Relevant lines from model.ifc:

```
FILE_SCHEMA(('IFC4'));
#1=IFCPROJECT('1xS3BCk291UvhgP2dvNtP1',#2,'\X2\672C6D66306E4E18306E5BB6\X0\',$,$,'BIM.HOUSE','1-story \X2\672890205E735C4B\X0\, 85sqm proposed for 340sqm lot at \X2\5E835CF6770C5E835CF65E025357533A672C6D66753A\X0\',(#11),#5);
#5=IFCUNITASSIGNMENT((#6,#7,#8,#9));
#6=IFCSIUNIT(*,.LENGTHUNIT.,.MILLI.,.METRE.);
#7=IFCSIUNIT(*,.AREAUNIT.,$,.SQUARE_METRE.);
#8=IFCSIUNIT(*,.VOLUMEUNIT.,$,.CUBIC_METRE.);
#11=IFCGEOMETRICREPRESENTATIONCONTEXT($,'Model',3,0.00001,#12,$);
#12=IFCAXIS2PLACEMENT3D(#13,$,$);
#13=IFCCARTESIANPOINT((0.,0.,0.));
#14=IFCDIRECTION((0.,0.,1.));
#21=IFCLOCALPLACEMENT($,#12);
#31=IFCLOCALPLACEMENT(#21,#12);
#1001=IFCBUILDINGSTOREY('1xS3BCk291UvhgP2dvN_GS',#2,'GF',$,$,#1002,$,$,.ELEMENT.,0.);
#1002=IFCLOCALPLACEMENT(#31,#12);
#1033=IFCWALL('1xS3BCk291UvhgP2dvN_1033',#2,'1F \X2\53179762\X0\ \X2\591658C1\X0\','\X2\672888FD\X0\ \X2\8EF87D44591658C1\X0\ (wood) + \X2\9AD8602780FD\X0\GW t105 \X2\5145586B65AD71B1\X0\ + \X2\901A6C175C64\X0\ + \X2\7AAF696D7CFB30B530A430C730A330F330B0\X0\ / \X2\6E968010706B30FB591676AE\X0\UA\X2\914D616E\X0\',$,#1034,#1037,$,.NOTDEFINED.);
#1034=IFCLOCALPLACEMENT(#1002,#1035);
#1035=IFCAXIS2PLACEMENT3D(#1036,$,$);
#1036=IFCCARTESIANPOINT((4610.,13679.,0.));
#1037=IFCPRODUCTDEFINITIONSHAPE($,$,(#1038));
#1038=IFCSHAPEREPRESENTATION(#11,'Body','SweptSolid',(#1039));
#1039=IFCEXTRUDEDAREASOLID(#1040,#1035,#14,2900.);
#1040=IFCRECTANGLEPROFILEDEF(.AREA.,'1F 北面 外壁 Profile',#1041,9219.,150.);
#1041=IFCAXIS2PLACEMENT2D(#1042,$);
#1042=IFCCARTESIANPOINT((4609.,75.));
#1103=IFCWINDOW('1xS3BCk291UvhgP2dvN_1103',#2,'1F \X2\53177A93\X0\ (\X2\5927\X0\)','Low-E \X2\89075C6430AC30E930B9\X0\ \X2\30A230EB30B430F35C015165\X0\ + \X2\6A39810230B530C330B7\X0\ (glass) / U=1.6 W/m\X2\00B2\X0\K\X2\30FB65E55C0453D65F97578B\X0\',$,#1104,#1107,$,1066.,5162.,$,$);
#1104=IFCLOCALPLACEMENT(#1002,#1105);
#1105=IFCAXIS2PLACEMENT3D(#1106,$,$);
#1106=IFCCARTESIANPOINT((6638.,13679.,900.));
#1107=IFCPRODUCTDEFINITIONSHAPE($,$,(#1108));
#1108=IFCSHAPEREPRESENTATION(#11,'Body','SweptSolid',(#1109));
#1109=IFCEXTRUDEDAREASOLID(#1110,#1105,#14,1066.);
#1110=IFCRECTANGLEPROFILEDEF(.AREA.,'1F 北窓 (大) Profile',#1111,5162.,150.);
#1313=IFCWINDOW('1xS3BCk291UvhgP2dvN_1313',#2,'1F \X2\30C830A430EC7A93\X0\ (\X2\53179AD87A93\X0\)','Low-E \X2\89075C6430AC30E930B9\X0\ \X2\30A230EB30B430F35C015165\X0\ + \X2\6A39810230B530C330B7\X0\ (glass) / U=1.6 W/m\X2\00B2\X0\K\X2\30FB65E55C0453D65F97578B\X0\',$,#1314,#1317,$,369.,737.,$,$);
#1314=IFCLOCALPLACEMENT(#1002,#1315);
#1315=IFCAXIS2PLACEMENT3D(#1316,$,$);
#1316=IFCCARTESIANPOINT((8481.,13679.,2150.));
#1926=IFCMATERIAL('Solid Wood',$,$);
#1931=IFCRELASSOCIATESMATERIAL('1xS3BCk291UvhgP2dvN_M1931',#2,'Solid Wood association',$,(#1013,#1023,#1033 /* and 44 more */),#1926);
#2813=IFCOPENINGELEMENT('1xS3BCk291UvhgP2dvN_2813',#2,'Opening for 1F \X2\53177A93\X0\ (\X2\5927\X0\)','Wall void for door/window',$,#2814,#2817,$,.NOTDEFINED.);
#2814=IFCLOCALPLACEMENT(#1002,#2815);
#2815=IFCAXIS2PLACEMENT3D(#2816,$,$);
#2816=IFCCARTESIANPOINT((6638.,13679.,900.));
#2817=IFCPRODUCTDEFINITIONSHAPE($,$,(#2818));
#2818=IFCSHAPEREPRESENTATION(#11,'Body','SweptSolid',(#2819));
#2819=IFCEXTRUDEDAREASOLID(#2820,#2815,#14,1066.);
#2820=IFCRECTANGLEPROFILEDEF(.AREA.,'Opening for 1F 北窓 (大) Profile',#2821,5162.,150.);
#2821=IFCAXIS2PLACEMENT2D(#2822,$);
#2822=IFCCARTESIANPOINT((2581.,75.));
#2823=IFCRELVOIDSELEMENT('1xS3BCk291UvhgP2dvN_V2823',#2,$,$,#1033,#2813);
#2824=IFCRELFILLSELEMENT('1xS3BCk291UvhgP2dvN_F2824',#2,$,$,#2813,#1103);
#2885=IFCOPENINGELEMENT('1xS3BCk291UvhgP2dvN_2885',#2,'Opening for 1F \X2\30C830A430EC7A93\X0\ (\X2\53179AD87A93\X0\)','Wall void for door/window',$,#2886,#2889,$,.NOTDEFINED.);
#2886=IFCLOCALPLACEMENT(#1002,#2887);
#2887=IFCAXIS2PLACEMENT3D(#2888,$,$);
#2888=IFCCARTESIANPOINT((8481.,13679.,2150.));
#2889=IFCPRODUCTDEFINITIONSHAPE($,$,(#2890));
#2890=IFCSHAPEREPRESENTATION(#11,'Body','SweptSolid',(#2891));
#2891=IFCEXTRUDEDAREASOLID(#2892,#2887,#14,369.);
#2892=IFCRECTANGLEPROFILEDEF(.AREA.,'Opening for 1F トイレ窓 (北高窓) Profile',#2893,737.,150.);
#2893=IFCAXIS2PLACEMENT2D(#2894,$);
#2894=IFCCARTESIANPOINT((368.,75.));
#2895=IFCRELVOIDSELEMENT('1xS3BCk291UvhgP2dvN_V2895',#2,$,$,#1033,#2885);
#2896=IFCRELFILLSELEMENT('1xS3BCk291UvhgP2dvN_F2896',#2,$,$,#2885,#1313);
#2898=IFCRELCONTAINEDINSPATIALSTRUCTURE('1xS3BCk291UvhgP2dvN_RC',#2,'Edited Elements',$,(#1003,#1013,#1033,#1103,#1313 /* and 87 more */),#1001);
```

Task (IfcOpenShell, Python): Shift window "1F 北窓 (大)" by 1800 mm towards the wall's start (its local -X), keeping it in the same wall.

```python
import ifcopenshell
import ifcopenshell.api.geometry
import ifcopenshell.util.placement
import ifcopenshell.util.unit

model = ifcopenshell.open("model.ifc")
unit_scale = ifcopenshell.util.unit.calculate_unit_scale(model)

window = model.by_guid("1xS3BCk291UvhgP2dvN_1103")
opening = window.FillsVoids[0].RelatingOpeningElement
wall = opening.VoidsElements[0].RelatingBuildingElement

wall_matrix = ifcopenshell.util.placement.get_local_placement(wall.ObjectPlacement)
shift = wall_matrix[:3, 0] * -1.8 / unit_scale
before = ifcopenshell.util.placement.get_local_placement(window.ObjectPlacement)[:3, 3].copy()

# The window is not placed relative to its opening, so move both.
for product in (opening, window):
    matrix = ifcopenshell.util.placement.get_local_placement(product.ObjectPlacement)
    matrix[:3, 3] += shift
    ifcopenshell.api.geometry.edit_object_placement(model, product=product, matrix=matrix, is_si=False)

after = ifcopenshell.util.placement.get_local_placement(window.ObjectPlacement)[:3, 3]
print("window moved by", (after - before).round(3) + 0.0)

model.write("model_edited.ifc")
```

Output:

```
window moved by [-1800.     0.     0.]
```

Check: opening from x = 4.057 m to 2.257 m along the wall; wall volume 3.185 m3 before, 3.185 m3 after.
